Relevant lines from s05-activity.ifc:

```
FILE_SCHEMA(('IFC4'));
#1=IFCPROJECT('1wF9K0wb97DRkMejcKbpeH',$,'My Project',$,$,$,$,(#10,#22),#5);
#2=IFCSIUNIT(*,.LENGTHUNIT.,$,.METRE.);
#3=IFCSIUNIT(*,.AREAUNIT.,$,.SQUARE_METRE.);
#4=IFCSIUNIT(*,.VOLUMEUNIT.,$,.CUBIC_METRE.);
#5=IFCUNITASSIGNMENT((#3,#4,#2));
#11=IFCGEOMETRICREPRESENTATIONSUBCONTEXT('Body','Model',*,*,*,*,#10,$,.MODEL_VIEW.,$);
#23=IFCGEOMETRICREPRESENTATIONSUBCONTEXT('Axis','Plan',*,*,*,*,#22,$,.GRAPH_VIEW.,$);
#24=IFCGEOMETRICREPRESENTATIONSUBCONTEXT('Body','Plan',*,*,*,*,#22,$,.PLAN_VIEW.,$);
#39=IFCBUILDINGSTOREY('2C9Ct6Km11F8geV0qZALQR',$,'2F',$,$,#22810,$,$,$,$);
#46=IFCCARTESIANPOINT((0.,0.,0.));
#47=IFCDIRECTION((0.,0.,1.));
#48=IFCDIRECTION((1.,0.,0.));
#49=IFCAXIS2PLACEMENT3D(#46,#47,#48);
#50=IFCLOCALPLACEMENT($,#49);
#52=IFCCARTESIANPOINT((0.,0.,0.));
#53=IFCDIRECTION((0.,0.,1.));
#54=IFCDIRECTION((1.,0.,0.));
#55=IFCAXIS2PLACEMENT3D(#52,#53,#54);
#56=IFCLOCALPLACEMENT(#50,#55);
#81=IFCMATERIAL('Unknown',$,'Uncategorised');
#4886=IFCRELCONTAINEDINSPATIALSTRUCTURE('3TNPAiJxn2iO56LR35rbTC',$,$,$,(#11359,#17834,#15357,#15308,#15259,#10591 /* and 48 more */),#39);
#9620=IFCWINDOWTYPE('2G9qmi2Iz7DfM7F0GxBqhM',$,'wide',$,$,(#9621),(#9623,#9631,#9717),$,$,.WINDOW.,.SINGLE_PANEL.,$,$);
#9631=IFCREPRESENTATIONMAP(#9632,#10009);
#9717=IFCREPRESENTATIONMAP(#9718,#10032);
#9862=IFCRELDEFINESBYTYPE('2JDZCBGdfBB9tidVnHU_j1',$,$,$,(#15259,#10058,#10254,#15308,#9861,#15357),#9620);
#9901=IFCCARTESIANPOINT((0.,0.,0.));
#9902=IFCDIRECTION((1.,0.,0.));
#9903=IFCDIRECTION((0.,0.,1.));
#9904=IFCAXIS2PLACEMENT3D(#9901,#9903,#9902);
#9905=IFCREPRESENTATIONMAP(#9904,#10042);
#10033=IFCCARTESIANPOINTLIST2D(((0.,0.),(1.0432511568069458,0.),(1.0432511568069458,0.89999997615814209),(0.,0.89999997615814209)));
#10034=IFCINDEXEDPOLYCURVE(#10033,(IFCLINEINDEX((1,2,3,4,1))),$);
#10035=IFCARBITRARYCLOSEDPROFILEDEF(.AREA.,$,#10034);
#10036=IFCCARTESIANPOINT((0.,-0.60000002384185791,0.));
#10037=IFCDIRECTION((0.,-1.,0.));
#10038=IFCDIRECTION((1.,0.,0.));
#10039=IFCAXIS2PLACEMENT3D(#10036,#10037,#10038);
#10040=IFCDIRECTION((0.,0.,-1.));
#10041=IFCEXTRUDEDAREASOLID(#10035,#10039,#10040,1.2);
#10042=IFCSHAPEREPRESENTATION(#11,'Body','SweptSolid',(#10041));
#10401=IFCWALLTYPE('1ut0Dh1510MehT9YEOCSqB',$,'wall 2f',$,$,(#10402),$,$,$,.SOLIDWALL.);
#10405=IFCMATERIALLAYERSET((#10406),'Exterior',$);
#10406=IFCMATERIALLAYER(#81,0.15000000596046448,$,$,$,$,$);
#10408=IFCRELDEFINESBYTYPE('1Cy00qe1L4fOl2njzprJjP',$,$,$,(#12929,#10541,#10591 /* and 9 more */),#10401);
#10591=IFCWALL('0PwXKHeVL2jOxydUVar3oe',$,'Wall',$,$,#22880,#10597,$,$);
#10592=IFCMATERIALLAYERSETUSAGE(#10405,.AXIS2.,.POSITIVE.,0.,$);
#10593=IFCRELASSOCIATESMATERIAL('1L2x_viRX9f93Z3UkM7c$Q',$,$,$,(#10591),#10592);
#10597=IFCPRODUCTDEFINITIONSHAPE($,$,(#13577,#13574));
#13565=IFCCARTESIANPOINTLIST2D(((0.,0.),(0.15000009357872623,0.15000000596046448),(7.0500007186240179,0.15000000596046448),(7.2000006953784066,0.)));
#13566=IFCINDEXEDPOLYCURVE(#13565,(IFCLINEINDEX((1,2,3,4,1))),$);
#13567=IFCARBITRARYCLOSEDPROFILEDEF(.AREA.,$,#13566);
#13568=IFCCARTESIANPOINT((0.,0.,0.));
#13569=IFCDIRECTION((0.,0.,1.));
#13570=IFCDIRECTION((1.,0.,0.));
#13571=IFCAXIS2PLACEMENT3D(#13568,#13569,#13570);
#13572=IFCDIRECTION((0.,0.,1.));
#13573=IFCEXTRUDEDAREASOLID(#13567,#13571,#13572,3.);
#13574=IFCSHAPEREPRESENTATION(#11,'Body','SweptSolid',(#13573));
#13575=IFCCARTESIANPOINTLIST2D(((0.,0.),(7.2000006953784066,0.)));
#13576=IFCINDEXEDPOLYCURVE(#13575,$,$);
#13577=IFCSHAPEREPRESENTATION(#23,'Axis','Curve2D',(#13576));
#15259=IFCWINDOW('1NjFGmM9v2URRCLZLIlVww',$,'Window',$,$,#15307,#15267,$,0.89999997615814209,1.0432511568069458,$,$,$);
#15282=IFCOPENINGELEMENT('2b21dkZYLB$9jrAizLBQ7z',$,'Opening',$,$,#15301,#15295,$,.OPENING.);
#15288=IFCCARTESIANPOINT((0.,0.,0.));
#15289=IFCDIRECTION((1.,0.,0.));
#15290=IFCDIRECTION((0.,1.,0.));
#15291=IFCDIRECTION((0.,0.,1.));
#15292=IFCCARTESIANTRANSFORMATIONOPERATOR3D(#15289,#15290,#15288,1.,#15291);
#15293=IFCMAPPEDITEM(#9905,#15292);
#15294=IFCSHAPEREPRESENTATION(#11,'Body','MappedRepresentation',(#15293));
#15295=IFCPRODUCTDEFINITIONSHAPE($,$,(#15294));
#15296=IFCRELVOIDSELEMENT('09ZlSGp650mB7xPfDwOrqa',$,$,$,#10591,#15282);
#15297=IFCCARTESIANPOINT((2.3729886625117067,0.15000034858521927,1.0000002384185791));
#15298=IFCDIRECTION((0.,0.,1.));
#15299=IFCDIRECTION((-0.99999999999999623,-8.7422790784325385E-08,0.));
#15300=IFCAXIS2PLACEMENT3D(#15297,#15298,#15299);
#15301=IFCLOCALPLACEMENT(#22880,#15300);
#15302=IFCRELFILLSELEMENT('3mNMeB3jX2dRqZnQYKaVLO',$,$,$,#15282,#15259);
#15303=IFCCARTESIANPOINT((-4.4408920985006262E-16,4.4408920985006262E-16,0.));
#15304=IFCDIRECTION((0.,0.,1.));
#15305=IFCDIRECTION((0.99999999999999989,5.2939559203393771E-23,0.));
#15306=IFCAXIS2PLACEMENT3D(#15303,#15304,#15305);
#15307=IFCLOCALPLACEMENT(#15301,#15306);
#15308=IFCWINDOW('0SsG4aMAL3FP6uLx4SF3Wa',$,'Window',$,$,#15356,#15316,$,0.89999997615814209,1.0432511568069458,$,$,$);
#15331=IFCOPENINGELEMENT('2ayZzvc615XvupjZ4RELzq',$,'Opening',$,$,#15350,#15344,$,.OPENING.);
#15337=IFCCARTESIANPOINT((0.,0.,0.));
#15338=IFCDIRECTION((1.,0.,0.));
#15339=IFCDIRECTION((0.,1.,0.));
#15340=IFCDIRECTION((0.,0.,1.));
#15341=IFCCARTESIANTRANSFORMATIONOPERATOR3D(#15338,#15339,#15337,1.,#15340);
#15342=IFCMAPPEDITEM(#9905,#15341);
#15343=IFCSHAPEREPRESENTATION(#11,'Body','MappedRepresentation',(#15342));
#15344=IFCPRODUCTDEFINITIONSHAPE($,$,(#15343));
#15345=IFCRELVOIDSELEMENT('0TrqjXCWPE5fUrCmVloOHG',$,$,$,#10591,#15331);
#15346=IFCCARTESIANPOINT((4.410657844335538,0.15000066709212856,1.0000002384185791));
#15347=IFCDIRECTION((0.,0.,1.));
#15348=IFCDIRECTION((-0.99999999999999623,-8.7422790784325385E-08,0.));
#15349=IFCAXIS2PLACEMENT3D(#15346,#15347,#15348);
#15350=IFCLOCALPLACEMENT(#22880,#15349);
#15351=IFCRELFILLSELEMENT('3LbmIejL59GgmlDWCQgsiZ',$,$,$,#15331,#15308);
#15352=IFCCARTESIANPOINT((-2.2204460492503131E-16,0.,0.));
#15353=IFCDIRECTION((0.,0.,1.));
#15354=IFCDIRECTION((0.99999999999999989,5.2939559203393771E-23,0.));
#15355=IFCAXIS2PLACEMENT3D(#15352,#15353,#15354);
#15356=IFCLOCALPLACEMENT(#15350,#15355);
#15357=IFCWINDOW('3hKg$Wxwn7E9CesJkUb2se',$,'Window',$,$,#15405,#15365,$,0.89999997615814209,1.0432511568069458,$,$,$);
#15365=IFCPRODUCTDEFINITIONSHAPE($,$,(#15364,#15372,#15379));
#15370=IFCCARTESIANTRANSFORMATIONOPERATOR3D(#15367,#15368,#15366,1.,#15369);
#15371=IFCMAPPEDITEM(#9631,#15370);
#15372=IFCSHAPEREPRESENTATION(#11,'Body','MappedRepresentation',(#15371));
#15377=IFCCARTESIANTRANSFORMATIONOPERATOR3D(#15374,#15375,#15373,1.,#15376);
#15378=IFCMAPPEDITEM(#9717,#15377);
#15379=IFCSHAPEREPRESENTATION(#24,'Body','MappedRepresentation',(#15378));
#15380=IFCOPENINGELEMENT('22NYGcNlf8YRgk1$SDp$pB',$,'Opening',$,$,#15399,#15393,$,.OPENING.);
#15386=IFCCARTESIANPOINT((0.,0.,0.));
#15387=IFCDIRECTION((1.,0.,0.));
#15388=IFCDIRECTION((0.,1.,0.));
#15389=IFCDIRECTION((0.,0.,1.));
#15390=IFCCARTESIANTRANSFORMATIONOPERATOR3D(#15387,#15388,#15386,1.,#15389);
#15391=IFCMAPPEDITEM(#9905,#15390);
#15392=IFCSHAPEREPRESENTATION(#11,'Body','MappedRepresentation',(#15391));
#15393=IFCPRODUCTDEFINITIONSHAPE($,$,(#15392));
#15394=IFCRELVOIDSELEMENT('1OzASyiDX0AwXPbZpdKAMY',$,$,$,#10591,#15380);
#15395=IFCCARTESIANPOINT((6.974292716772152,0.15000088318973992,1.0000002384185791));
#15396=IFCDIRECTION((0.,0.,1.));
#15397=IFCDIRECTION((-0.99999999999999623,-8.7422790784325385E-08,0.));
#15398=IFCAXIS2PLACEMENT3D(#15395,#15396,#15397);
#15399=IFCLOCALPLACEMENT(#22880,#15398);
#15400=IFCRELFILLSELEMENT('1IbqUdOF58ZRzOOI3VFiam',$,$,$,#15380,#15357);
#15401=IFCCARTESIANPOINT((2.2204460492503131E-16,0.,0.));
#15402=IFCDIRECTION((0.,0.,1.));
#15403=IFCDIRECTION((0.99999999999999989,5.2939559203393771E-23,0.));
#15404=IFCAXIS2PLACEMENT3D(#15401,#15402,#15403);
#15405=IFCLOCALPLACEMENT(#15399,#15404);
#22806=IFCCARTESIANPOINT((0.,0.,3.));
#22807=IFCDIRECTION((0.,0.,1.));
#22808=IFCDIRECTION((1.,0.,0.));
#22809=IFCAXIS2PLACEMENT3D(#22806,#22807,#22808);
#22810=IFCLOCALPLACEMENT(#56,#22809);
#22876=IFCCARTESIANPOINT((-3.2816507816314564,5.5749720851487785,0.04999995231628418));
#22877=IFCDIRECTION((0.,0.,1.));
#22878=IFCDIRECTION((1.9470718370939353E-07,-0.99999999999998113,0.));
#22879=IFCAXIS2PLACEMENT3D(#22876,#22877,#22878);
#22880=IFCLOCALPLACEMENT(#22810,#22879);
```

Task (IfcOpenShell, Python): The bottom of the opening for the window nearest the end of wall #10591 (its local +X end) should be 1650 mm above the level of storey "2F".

```python
import numpy as np
import ifcopenshell
import ifcopenshell.api.geometry
import ifcopenshell.geom
import ifcopenshell.util.element
import ifcopenshell.util.placement
import ifcopenshell.util.shape
import ifcopenshell.util.unit

model = ifcopenshell.open("s05-activity.ifc")
unit_scale = ifcopenshell.util.unit.calculate_unit_scale(model)

window = model.by_guid("3hKg$Wxwn7E9CesJkUb2se")
opening = window.FillsVoids[0].RelatingOpeningElement
storey = ifcopenshell.util.element.get_container(window, ifc_class="IfcBuildingStorey")
level = ifcopenshell.util.placement.get_local_placement(storey.ObjectPlacement)[2, 3]

# The opening's origin need not be at the sill, so measure its lowest point.
shape = ifcopenshell.geom.create_shape(ifcopenshell.geom.settings(), opening)
bottom = ifcopenshell.util.shape.get_shape_bottom_elevation(shape, shape.geometry) / unit_scale
dz = level + 1.65 / unit_scale - bottom

shift = np.array([0.0, 0.0, dz])
# The window is placed relative to its opening, so it follows when the opening moves.
matrix = ifcopenshell.util.placement.get_local_placement(opening.ObjectPlacement)
matrix[:3, 3] += shift
ifcopenshell.api.geometry.edit_object_placement(
    model, product=opening, matrix=matrix, is_si=False, should_transform_children=True
)

print(f"moved by {dz * unit_scale:+.3f} m")

model.write("s05-activity-out.ifc")
```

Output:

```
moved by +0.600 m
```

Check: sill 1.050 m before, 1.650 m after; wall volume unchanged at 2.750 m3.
